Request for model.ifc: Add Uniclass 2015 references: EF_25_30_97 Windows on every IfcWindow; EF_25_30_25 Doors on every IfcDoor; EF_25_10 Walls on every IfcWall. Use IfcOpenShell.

First a look at what the model holds.

```python
import ifcopenshell

model = ifcopenshell.open("model.ifc")
print(model.schema)
print("classifications:", [c.Name for c in model.by_type("IfcClassification")])
for ifc_class in ("IfcDoor", "IfcRoof", "IfcStair", "IfcWall", "IfcWindow"):
    print(ifc_class, len(model.by_type(ifc_class)))
```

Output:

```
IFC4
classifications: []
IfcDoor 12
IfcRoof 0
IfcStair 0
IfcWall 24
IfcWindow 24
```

```python
import ifcopenshell
import ifcopenshell.api.classification

model = ifcopenshell.open("model.ifc")

system = ifcopenshell.api.classification.add_classification(model, classification="Uniclass 2015")

codes = {
    "IfcWindow": ("EF_25_30_97", "Windows"),
    "IfcDoor": ("EF_25_30_25", "Doors"),
    "IfcWall": ("EF_25_10", "Walls"),
}
for ifc_class, (code, name) in codes.items():
    products = model.by_type(ifc_class)
    ifcopenshell.api.classification.add_reference(
        model, products=products, classification=system, identification=code, name=name
    )
    print(code, len(products))

model.write("model_updated.ifc")
```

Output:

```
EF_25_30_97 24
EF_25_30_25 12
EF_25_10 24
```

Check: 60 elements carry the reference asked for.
